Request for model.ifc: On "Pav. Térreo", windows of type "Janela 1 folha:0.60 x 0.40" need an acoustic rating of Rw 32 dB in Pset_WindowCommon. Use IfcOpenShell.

First a look at what the model holds.

```python
import ifcopenshell
import ifcopenshell.util.element

model = ifcopenshell.open("model.ifc")
print(model.schema)
storey = next(s for s in model.by_type("IfcBuildingStorey") if s.Name == "Pav. Térreo")
windows = [e for e in ifcopenshell.util.element.get_decomposition(storey) if e.is_a("IfcWindow")]
seen = {}
for e in windows:
    element_type = ifcopenshell.util.element.get_type(e)
    key = (element_type.Name if element_type != e and element_type else None, ifcopenshell.util.element.get_pset(e, "Pset_WindowCommon", "AcousticRating"))
    seen[key] = seen.get(key, 0) + 1
for (name, value), count in sorted(seen.items(), key=str):
    print(count, "x", name, "|", value)
```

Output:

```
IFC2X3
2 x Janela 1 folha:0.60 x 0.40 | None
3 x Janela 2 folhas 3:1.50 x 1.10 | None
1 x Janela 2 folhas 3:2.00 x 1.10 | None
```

```python
import ifcopenshell
import ifcopenshell.api.pset
import ifcopenshell.util.element

model = ifcopenshell.open("model.ifc")

storey = next(s for s in model.by_type("IfcBuildingStorey") if s.Name == "Pav. Térreo")
windows = [e for e in ifcopenshell.util.element.get_decomposition(storey) if e.is_a("IfcWindow")]

count = 0
for e in windows:
    element_type = ifcopenshell.util.element.get_type(e)
    if element_type in (None, e) or element_type.Name != "Janela 1 folha:0.60 x 0.40":
        continue
    # add_pset returns the element's existing set when there is one.
    pset = ifcopenshell.api.pset.add_pset(model, product=e, name="Pset_WindowCommon")
    ifcopenshell.api.pset.edit_pset(model, pset=pset, properties={"AcousticRating": "Rw 32 dB"})
    count += 1

print(count, "windows updated")

model.write("model_rev.ifc")
```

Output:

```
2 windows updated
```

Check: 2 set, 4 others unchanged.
